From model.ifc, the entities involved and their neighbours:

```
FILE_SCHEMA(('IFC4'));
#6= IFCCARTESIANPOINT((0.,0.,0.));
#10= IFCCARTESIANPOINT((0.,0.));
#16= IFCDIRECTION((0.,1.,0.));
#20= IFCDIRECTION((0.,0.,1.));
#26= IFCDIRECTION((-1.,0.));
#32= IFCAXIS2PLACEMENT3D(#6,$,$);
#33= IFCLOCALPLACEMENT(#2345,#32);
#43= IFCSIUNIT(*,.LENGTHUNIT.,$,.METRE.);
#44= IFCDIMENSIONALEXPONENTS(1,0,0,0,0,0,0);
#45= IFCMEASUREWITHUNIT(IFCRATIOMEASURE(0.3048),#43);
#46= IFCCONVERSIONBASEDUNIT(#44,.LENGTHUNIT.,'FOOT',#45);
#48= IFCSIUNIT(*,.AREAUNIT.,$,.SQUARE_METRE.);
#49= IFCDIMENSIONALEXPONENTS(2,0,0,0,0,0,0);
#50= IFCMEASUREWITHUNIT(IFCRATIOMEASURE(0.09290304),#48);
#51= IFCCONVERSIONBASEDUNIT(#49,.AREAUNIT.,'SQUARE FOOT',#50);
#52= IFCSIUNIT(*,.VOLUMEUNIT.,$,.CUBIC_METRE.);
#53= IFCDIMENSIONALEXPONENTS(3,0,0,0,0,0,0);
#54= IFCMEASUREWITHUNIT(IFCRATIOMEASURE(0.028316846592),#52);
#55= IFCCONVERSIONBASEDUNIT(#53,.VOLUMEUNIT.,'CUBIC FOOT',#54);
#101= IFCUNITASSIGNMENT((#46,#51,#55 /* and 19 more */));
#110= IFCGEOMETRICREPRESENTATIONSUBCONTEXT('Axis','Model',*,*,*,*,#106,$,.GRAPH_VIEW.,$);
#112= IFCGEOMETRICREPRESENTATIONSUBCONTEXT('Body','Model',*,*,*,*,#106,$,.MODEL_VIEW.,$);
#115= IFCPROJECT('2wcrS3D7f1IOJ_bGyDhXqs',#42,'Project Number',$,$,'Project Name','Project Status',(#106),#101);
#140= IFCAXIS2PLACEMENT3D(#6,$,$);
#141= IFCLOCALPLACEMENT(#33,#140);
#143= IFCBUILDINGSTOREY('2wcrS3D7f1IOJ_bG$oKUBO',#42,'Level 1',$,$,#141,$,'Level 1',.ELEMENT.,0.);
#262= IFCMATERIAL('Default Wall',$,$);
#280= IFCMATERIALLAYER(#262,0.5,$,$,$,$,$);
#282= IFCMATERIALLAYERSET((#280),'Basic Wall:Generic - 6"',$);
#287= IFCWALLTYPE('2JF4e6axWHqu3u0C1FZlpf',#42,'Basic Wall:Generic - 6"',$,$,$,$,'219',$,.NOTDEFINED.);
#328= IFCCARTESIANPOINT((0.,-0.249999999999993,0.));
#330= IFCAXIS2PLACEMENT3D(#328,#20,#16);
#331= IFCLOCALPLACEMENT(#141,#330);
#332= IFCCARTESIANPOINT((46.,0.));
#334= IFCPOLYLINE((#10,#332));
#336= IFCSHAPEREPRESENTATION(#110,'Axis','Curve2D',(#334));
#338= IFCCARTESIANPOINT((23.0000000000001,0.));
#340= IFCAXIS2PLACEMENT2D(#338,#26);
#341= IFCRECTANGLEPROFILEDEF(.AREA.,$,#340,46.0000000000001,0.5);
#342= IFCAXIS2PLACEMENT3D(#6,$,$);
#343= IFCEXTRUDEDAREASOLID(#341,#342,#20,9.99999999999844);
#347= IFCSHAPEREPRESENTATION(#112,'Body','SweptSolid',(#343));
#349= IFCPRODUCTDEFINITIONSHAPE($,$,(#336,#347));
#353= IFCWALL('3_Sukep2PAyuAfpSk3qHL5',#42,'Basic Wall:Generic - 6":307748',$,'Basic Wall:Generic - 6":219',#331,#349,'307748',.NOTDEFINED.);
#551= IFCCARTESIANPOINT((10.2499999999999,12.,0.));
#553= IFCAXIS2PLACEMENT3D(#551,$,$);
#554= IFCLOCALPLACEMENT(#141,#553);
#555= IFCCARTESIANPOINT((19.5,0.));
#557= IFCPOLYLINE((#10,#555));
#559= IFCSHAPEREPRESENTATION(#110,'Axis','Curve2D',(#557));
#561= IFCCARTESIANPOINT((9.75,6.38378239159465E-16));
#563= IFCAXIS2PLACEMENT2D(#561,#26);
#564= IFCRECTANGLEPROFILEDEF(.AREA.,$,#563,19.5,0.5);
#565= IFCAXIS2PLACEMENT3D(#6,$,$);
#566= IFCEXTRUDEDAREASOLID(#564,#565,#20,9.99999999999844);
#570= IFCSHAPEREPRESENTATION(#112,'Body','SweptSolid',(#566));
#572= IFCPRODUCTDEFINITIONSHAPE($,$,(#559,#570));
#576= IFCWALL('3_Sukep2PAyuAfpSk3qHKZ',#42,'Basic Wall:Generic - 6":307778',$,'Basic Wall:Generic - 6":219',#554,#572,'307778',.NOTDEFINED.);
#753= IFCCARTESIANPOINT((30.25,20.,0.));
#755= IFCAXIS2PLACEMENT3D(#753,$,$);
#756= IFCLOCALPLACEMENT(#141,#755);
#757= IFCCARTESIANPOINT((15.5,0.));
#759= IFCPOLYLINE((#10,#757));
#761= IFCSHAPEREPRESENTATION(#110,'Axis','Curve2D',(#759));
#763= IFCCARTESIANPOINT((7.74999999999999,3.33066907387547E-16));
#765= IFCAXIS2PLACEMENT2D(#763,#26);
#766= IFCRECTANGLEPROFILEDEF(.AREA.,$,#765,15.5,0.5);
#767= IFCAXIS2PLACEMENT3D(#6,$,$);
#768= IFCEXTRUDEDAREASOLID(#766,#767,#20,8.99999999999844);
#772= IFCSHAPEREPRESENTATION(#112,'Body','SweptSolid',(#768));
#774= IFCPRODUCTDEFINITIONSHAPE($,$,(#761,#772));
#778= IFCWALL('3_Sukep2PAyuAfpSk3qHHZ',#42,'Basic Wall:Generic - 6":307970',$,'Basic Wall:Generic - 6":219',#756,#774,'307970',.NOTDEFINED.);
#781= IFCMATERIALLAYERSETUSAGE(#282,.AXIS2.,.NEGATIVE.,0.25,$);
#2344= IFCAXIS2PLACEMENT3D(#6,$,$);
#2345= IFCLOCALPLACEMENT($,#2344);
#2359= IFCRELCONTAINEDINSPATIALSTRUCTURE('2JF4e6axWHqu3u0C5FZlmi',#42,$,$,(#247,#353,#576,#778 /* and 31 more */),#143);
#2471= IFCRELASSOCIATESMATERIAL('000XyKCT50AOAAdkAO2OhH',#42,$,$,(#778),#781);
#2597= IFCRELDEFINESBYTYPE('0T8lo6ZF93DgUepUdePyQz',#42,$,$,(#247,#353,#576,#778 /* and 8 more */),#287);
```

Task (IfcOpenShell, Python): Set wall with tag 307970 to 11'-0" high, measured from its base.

```python
import ifcopenshell
import ifcopenshell.geom
import ifcopenshell.util.representation
import ifcopenshell.util.shape
import ifcopenshell.util.unit

model = ifcopenshell.open("model.ifc")
unit_scale = ifcopenshell.util.unit.calculate_unit_scale(model)
settings = ifcopenshell.geom.settings()


def volume(element):
    """Net volume in cubic metres, openings subtracted."""
    shape = ifcopenshell.geom.create_shape(settings, element)
    return ifcopenshell.util.shape.get_volume(shape.geometry)


wall = model.by_guid("3_Sukep2PAyuAfpSk3qHHZ")
before = volume(wall)

body = ifcopenshell.util.representation.get_representation(wall, "Model", "Body")
solid = body.Items[0]
old_height = solid.Depth
solid.Depth = 132 * 0.0254 / unit_scale
after = volume(wall)

print(f"height {old_height:g} -> {solid.Depth:g}, volume {before:.3f} -> {after:.3f} m3")

model.write("model_updated.ifc")
```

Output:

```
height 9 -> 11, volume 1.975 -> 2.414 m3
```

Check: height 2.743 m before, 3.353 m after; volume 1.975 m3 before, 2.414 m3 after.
